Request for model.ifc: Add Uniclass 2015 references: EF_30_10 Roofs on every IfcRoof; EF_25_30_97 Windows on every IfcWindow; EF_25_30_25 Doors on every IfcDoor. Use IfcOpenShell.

First a look at what the model holds.

```python
import ifcopenshell

model = ifcopenshell.open("model.ifc")
print(model.schema)
print("classifications:", [c.Name for c in model.by_type("IfcClassification")])
for ifc_class in ("IfcDoor", "IfcRoof", "IfcStair", "IfcWall", "IfcWindow"):
    print(ifc_class, len(model.by_type(ifc_class)))
```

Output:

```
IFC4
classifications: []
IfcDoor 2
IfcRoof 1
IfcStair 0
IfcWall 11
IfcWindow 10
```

```python
import ifcopenshell
import ifcopenshell.api.classification

model = ifcopenshell.open("model.ifc")

system = ifcopenshell.api.classification.add_classification(model, classification="Uniclass 2015")

codes = {
    "IfcRoof": ("EF_30_10", "Roofs"),
    "IfcWindow": ("EF_25_30_97", "Windows"),
    "IfcDoor": ("EF_25_30_25", "Doors"),
}
for ifc_class, (code, name) in codes.items():
    products = model.by_type(ifc_class)
    ifcopenshell.api.classification.add_reference(
        model, products=products, classification=system, identification=code, name=name
    )
    print(code, len(products))

model.write("model_edited.ifc")
```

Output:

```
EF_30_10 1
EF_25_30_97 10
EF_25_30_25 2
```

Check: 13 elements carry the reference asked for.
